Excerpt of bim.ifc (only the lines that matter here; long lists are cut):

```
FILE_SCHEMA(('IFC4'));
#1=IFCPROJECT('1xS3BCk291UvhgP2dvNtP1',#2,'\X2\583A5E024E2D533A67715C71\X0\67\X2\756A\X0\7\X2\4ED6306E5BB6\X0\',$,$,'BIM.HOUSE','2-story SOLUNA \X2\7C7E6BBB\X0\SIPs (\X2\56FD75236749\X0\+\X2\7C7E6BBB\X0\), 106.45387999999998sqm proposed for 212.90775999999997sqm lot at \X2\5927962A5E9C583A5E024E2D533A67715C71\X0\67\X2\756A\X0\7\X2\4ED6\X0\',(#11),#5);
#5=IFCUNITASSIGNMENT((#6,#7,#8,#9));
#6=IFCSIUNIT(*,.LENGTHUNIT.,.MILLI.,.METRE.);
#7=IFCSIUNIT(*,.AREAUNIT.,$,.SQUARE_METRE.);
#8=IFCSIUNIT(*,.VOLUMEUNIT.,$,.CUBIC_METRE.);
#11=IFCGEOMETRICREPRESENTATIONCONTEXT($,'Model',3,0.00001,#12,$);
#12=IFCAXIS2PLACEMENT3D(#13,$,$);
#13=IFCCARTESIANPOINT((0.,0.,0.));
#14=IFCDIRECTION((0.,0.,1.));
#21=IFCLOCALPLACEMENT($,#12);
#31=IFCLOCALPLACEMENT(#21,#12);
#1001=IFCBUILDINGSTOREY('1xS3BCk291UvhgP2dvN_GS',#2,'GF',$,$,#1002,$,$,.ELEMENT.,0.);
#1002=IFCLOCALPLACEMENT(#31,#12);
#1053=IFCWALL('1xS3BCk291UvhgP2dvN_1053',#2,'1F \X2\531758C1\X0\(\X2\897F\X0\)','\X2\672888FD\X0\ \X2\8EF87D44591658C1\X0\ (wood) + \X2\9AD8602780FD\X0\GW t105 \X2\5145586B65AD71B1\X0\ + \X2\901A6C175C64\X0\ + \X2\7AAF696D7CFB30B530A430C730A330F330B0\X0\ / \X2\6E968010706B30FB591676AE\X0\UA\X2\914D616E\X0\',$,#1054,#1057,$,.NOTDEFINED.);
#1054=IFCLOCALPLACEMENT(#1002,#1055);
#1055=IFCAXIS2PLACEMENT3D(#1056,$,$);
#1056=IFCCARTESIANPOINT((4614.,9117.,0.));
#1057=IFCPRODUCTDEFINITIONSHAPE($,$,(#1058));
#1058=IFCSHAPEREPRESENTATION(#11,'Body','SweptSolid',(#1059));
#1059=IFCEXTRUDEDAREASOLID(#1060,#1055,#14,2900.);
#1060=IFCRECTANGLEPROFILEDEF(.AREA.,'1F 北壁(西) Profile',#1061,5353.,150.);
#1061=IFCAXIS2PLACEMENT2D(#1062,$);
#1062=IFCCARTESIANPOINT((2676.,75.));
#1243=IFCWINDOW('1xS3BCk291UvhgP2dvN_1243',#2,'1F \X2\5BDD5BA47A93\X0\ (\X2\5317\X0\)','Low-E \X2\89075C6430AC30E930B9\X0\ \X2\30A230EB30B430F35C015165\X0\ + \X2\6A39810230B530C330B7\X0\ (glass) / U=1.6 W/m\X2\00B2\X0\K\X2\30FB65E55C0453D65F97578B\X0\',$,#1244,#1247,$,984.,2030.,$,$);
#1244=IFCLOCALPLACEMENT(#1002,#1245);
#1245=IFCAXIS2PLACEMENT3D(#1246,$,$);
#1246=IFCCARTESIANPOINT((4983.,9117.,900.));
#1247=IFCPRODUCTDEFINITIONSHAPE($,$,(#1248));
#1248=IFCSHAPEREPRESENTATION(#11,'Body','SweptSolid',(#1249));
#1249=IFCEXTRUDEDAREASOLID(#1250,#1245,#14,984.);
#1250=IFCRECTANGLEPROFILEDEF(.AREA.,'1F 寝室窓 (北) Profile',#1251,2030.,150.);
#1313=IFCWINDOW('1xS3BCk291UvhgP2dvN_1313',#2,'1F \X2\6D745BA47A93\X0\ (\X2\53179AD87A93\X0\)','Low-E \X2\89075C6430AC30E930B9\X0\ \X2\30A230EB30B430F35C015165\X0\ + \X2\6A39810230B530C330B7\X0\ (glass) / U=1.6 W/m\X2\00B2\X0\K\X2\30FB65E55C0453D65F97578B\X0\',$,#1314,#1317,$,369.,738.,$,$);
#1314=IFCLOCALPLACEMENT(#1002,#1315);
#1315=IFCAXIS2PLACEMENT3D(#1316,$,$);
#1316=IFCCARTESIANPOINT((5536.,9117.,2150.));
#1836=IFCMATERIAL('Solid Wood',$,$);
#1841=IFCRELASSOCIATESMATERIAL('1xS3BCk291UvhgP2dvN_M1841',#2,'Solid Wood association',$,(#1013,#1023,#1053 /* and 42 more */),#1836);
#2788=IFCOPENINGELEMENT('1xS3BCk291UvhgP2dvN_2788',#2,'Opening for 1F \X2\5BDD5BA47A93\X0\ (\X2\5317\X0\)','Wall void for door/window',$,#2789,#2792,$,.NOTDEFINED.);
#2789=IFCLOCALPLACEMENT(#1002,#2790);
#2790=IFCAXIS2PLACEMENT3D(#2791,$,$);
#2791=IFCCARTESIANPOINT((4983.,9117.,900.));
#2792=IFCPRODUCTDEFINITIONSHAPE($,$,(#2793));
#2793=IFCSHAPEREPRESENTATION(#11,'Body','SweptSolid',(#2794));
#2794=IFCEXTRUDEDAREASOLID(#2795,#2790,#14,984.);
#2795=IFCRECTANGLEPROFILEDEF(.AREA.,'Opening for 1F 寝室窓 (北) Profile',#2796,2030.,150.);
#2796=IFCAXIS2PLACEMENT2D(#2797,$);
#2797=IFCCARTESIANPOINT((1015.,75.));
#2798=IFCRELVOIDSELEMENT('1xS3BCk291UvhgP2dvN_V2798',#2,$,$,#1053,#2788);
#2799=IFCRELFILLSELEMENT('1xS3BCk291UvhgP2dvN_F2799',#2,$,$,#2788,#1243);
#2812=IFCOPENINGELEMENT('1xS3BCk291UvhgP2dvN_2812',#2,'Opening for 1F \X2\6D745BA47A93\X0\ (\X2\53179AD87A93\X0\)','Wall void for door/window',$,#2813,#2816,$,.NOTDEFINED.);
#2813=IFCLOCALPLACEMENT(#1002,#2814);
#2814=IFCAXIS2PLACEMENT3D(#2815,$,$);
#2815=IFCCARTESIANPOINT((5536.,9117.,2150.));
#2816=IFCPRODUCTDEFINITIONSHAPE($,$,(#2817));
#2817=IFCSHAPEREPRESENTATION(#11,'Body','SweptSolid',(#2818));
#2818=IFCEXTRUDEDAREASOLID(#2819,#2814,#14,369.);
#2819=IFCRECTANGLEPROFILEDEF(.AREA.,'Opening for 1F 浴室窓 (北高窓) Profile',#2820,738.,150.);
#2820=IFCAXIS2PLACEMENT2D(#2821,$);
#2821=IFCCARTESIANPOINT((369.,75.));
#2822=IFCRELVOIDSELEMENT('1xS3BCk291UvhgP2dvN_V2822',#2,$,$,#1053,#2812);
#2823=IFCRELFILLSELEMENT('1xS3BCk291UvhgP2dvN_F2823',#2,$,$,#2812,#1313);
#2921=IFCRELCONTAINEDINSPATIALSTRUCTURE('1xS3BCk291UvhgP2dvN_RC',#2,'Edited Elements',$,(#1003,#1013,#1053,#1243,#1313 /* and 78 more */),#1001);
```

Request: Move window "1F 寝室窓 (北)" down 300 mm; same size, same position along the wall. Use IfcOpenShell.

```python
import numpy as np
import ifcopenshell
import ifcopenshell.api.geometry
import ifcopenshell.util.placement
import ifcopenshell.util.unit

model = ifcopenshell.open("bim.ifc")
unit_scale = ifcopenshell.util.unit.calculate_unit_scale(model)

window = model.by_guid("1xS3BCk291UvhgP2dvN_1243")
opening = window.FillsVoids[0].RelatingOpeningElement
dz = -300.0

shift = np.array([0.0, 0.0, dz])
# The window is not placed relative to its opening, so move both.
for product in (opening, window):
    matrix = ifcopenshell.util.placement.get_local_placement(product.ObjectPlacement)
    matrix[:3, 3] += shift
    ifcopenshell.api.geometry.edit_object_placement(model, product=product, matrix=matrix, is_si=False)

print(f"moved by {dz * unit_scale:+.3f} m")

model.write("bim_v2.ifc")
```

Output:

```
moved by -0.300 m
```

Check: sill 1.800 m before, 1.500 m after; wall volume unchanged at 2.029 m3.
